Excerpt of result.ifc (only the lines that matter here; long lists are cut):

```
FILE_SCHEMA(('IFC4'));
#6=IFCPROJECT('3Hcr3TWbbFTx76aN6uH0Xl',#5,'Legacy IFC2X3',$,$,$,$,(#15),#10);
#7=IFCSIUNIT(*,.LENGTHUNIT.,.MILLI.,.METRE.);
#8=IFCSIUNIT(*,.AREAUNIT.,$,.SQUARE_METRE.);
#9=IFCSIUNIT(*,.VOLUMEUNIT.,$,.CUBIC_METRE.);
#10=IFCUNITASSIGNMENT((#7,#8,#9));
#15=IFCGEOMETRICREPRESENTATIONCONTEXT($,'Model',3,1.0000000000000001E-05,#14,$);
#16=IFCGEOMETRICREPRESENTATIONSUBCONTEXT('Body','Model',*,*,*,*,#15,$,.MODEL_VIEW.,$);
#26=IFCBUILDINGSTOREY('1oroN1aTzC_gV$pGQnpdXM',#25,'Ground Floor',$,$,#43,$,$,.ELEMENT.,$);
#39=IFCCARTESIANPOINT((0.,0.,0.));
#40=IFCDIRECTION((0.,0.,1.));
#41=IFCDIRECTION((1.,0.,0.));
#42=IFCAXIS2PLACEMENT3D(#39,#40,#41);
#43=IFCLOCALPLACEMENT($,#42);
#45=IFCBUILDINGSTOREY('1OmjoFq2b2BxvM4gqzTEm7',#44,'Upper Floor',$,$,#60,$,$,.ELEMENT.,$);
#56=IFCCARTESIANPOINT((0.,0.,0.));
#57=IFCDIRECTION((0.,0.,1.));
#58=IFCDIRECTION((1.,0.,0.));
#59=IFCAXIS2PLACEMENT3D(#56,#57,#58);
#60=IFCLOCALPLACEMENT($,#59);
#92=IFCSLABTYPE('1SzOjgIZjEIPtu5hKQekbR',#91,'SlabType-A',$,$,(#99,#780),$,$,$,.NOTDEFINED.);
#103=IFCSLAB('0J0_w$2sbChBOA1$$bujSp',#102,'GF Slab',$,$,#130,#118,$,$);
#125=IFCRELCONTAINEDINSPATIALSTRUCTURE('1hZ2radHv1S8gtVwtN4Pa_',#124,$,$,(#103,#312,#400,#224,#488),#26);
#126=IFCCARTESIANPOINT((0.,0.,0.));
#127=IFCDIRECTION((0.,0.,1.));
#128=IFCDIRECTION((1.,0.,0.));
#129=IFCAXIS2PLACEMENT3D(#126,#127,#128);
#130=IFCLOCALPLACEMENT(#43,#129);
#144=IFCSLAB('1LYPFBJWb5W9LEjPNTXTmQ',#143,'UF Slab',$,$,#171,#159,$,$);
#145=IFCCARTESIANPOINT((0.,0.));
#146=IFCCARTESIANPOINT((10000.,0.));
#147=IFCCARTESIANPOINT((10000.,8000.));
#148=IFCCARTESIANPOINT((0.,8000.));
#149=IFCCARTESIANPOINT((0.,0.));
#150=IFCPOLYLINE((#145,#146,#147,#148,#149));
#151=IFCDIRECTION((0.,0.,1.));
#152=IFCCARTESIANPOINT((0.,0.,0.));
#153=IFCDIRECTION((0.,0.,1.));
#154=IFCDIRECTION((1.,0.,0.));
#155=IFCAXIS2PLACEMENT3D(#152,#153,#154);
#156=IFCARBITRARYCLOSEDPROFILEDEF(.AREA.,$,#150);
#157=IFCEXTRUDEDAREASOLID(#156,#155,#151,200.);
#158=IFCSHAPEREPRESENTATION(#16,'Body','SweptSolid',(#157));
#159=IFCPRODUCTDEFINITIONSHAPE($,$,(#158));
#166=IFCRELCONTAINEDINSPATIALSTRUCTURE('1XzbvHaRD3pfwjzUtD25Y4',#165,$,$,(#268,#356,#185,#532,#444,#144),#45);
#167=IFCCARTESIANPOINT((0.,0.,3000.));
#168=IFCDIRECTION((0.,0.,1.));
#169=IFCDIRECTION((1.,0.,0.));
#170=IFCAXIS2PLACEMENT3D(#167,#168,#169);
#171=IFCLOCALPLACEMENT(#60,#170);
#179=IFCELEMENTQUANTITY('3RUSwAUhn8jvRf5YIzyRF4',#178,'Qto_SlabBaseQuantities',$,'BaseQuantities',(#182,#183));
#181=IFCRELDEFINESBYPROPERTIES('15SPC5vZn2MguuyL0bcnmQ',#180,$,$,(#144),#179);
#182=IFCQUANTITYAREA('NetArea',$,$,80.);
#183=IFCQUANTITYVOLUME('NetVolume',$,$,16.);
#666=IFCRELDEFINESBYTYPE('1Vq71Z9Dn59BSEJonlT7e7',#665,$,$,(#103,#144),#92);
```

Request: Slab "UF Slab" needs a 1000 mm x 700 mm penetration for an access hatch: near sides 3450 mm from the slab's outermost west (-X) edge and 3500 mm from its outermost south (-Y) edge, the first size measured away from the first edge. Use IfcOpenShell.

```python
import numpy as np
import ifcopenshell
import ifcopenshell.api.feature
import ifcopenshell.api.geometry
import ifcopenshell.api.pset
import ifcopenshell.api.root
import ifcopenshell.geom
import ifcopenshell.util.element
import ifcopenshell.util.placement
import ifcopenshell.util.representation
import ifcopenshell.util.shape
import ifcopenshell.util.unit

model = ifcopenshell.open("result.ifc")
unit_scale = ifcopenshell.util.unit.calculate_unit_scale(model)
area_scale = ifcopenshell.util.unit.calculate_unit_scale(model, "AREAUNIT")
volume_scale = ifcopenshell.util.unit.calculate_unit_scale(model, "VOLUMEUNIT")
settings = ifcopenshell.geom.settings()


def volume(element):
    """Net volume in cubic metres, openings subtracted."""
    shape = ifcopenshell.geom.create_shape(settings, element)
    return ifcopenshell.util.shape.get_volume(shape.geometry)


slab = model.by_guid("1LYPFBJWb5W9LEjPNTXTmQ")
before = volume(slab)

# Extent in the slab's own axes, in metres. The edges named are its -X and -Y sides.
slab_shape = ifcopenshell.geom.create_shape(settings, slab)
vertices = ifcopenshell.util.shape.get_vertices(slab_shape.geometry)
x_min, y_min, bottom = vertices.min(axis=0)
top = vertices[:, 2].max()

opening = ifcopenshell.api.root.create_entity(model, ifc_class="IfcOpeningElement", name="Access hatch opening", predefined_type="OPENING")
context = ifcopenshell.util.representation.get_context(model, "Model", "Body", "MODEL_VIEW")
width, depth = 1, 0.7
outline = [(0.0, 0.0), (width, 0.0), (width, depth), (0.0, depth), (0.0, 0.0)]
# Overshoot both faces by 50 mm so the cut is clean.
shape = ifcopenshell.api.geometry.add_slab_representation(
    model, context=context, depth=top - bottom + 0.1, polyline=outline
)
ifcopenshell.api.geometry.assign_representation(model, product=opening, representation=shape)

matrix = ifcopenshell.util.placement.get_local_placement(slab.ObjectPlacement)
matrix[:, 3] = matrix @ np.append(np.array([x_min + 3.45, y_min + 3.5, bottom - 0.05]) / unit_scale, 1.0)
ifcopenshell.api.geometry.edit_object_placement(model, product=opening, matrix=matrix, is_si=False)
ifcopenshell.api.feature.add_feature(model, feature=opening, element=slab)

after = volume(slab)

# Update the slab's stored quantities.
qto = model.by_id(ifcopenshell.util.element.get_pset(slab, "Qto_SlabBaseQuantities", should_inherit=False)["id"])
ifcopenshell.api.pset.edit_qto(model, qto=qto, properties={
    "NetArea": after / (top - bottom) / area_scale,
    "NetVolume": after / volume_scale,
})

print(f"slab volume {before:.3f} -> {after:.3f} m3")

model.write("result_v2.ifc")
```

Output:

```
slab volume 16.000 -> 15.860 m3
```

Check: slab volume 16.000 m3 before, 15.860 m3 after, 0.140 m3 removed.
